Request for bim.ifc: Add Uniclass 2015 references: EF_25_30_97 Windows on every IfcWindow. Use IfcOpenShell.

First a look at what the model holds.

```python
import ifcopenshell

model = ifcopenshell.open("bim.ifc")
print(model.schema)
print("classifications:", [c.Name for c in model.by_type("IfcClassification")])
for ifc_class in ("IfcDoor", "IfcRoof", "IfcStair", "IfcWall", "IfcWindow"):
    print(ifc_class, len(model.by_type(ifc_class)))
```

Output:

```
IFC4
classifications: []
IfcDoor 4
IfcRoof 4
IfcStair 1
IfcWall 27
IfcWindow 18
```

```python
import ifcopenshell
import ifcopenshell.api.classification

model = ifcopenshell.open("bim.ifc")

system = ifcopenshell.api.classification.add_classification(model, classification="Uniclass 2015")

codes = {
    "IfcWindow": ("EF_25_30_97", "Windows"),
}
for ifc_class, (code, name) in codes.items():
    products = model.by_type(ifc_class)
    ifcopenshell.api.classification.add_reference(
        model, products=products, classification=system, identification=code, name=name
    )
    print(code, len(products))

model.write("bim_v2.ifc")
```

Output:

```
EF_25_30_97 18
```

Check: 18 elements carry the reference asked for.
